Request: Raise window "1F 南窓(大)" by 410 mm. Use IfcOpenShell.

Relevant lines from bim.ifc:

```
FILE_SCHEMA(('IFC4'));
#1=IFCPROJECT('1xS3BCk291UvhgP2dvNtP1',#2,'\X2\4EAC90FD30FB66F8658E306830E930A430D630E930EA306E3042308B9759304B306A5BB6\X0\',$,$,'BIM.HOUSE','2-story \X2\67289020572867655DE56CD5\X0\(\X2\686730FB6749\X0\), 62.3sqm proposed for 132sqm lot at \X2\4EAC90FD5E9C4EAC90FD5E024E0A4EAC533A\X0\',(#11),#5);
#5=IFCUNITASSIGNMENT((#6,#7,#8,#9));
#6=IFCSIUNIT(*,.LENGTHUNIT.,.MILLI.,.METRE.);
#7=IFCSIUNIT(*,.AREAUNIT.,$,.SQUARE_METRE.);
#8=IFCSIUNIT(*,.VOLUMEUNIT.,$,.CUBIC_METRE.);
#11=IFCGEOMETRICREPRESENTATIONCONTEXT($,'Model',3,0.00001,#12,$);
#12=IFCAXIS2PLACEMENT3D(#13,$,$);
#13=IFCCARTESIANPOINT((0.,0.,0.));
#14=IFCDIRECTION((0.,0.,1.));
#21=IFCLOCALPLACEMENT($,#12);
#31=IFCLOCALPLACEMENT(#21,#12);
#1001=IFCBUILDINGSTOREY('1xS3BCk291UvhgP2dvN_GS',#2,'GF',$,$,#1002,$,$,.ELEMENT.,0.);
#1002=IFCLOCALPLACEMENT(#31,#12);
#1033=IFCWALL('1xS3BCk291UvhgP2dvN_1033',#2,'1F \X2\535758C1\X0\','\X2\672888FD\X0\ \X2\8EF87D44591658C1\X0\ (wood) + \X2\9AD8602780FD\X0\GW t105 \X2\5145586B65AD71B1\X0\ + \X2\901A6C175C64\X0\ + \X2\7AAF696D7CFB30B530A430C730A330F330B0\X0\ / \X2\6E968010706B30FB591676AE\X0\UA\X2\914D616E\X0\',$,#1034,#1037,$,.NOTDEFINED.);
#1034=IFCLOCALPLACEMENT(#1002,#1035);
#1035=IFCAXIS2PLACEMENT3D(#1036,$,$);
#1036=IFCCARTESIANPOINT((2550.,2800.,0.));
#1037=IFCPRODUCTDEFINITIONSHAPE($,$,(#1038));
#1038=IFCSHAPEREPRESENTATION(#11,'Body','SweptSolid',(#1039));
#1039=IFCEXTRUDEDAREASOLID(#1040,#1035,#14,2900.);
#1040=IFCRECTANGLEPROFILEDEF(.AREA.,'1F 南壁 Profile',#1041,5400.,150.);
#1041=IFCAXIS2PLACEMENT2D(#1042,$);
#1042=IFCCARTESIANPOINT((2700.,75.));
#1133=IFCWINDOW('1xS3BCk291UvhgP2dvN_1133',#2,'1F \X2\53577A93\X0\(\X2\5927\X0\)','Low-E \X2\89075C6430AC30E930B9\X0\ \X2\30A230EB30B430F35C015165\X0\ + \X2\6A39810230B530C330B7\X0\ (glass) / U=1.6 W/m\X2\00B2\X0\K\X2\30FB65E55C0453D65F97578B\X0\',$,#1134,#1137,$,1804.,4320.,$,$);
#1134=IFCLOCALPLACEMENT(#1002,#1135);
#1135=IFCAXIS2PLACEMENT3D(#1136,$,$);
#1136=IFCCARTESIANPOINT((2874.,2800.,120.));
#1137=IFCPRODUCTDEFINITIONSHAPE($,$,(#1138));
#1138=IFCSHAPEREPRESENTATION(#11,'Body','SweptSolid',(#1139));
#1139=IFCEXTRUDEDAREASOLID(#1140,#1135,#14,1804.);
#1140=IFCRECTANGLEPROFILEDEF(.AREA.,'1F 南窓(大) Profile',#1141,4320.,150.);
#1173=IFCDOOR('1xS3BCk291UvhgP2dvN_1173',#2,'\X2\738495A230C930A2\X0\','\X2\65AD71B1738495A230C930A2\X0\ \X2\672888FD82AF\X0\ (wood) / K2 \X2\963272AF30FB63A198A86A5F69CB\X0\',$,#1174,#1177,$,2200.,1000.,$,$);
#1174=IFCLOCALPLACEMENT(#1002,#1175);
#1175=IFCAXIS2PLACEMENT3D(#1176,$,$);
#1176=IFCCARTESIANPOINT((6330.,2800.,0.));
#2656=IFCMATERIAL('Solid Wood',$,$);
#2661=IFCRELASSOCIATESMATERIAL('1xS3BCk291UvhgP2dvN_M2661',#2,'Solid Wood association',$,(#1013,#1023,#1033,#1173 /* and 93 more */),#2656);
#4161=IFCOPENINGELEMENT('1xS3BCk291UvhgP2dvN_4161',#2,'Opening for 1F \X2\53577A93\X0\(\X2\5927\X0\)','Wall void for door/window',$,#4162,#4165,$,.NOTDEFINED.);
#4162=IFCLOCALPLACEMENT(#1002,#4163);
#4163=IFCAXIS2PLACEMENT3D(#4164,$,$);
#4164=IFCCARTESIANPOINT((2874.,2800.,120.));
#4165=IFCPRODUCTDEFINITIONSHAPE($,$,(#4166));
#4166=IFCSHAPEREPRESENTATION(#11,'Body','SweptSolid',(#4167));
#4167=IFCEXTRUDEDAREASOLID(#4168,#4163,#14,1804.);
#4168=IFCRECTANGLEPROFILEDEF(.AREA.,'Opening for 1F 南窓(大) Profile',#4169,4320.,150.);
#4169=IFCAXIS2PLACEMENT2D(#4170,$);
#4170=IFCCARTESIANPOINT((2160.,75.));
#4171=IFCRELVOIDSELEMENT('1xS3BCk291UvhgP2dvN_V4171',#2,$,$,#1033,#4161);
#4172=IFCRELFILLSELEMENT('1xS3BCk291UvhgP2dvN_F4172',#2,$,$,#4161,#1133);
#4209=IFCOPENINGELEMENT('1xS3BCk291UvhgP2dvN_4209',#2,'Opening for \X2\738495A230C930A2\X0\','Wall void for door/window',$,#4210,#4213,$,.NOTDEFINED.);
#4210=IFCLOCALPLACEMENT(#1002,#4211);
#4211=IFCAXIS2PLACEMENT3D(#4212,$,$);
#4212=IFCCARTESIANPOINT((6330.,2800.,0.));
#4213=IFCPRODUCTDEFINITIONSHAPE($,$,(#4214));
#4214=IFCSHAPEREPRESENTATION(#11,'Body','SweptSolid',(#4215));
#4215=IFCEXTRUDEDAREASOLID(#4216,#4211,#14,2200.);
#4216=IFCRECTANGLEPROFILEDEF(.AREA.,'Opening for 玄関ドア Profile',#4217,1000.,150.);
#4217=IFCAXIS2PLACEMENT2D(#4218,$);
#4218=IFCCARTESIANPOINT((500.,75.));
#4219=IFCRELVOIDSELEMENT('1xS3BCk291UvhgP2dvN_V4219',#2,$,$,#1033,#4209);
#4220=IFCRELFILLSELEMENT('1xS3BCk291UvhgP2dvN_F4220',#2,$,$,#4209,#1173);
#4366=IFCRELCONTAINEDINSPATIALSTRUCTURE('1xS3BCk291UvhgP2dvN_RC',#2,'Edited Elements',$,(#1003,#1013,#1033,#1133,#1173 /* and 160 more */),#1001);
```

```python
import numpy as np
import ifcopenshell
import ifcopenshell.api.geometry
import ifcopenshell.util.placement
import ifcopenshell.util.unit

model = ifcopenshell.open("bim.ifc")
unit_scale = ifcopenshell.util.unit.calculate_unit_scale(model)

window = model.by_id(1133)
opening = window.FillsVoids[0].RelatingOpeningElement
dz = 410.0

shift = np.array([0.0, 0.0, dz])
# The window is not placed relative to its opening, so move both.
for product in (opening, window):
    matrix = ifcopenshell.util.placement.get_local_placement(product.ObjectPlacement)
    matrix[:3, 3] += shift
    ifcopenshell.api.geometry.edit_object_placement(model, product=product, matrix=matrix, is_si=False)

print(f"moved by {dz * unit_scale:+.3f} m")

model.write("bim_edited.ifc")
```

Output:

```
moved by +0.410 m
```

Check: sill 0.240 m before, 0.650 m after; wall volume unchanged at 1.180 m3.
